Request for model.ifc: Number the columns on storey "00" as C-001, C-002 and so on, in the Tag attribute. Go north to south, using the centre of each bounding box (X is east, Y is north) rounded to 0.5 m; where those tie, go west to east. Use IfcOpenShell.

First a look at what the model holds.

```python
import ifcopenshell
import ifcopenshell.util.element
import ifcopenshell.util.placement

model = ifcopenshell.open("model.ifc")
print(model.schema)
storey = next(s for s in model.by_type("IfcBuildingStorey") if s.Name == "00")
columns = [e for e in ifcopenshell.util.element.get_decomposition(storey) if e.is_a("IfcColumn")]
for e in sorted(columns, key=lambda e: e.id()):
    origin = ifcopenshell.util.placement.get_local_placement(e.ObjectPlacement)[:3, 3]
    print(e.id(), e.Tag, e.Name, origin.round(2) + 0.0, sep=" | ")
```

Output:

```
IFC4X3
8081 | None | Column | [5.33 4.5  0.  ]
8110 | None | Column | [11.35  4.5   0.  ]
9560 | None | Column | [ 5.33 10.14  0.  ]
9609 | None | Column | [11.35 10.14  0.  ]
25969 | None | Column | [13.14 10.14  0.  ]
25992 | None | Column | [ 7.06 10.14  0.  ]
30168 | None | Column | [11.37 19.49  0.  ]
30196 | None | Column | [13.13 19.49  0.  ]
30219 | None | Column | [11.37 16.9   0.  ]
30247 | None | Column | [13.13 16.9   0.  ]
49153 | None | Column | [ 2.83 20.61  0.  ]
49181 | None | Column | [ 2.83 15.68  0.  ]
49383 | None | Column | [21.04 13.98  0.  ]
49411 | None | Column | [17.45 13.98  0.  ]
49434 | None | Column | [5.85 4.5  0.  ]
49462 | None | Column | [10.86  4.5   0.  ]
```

```python
import ifcopenshell
import ifcopenshell.geom
import ifcopenshell.util.element
import ifcopenshell.util.shape

model = ifcopenshell.open("model.ifc")
settings = ifcopenshell.geom.settings()
settings.set("use-world-coords", True)


def centre(element):
    shape = ifcopenshell.geom.create_shape(settings, element)
    return ifcopenshell.util.shape.get_bbox_centroid(shape.geometry)


storey = next(s for s in model.by_type("IfcBuildingStorey") if s.Name == "00")
columns = [e for e in ifcopenshell.util.element.get_decomposition(storey) if e.is_a("IfcColumn")]

# Insertion points can sit at a corner or the storey origin, so sort by the geometry (in metres).
centres = {e: centre(e) for e in columns}
columns.sort(key=lambda e: (-round(centres[e][1] / 0.5), centres[e][0]))

for i, e in enumerate(columns, start=1):
    number = f"C-0{i:02d}"
    e.Tag = number
    print(e.id(), number)

model.write("model_edited.ifc")
```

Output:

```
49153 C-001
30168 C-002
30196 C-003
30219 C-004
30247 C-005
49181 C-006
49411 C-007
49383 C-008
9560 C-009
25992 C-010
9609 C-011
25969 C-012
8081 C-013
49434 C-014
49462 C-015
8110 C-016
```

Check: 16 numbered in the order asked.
